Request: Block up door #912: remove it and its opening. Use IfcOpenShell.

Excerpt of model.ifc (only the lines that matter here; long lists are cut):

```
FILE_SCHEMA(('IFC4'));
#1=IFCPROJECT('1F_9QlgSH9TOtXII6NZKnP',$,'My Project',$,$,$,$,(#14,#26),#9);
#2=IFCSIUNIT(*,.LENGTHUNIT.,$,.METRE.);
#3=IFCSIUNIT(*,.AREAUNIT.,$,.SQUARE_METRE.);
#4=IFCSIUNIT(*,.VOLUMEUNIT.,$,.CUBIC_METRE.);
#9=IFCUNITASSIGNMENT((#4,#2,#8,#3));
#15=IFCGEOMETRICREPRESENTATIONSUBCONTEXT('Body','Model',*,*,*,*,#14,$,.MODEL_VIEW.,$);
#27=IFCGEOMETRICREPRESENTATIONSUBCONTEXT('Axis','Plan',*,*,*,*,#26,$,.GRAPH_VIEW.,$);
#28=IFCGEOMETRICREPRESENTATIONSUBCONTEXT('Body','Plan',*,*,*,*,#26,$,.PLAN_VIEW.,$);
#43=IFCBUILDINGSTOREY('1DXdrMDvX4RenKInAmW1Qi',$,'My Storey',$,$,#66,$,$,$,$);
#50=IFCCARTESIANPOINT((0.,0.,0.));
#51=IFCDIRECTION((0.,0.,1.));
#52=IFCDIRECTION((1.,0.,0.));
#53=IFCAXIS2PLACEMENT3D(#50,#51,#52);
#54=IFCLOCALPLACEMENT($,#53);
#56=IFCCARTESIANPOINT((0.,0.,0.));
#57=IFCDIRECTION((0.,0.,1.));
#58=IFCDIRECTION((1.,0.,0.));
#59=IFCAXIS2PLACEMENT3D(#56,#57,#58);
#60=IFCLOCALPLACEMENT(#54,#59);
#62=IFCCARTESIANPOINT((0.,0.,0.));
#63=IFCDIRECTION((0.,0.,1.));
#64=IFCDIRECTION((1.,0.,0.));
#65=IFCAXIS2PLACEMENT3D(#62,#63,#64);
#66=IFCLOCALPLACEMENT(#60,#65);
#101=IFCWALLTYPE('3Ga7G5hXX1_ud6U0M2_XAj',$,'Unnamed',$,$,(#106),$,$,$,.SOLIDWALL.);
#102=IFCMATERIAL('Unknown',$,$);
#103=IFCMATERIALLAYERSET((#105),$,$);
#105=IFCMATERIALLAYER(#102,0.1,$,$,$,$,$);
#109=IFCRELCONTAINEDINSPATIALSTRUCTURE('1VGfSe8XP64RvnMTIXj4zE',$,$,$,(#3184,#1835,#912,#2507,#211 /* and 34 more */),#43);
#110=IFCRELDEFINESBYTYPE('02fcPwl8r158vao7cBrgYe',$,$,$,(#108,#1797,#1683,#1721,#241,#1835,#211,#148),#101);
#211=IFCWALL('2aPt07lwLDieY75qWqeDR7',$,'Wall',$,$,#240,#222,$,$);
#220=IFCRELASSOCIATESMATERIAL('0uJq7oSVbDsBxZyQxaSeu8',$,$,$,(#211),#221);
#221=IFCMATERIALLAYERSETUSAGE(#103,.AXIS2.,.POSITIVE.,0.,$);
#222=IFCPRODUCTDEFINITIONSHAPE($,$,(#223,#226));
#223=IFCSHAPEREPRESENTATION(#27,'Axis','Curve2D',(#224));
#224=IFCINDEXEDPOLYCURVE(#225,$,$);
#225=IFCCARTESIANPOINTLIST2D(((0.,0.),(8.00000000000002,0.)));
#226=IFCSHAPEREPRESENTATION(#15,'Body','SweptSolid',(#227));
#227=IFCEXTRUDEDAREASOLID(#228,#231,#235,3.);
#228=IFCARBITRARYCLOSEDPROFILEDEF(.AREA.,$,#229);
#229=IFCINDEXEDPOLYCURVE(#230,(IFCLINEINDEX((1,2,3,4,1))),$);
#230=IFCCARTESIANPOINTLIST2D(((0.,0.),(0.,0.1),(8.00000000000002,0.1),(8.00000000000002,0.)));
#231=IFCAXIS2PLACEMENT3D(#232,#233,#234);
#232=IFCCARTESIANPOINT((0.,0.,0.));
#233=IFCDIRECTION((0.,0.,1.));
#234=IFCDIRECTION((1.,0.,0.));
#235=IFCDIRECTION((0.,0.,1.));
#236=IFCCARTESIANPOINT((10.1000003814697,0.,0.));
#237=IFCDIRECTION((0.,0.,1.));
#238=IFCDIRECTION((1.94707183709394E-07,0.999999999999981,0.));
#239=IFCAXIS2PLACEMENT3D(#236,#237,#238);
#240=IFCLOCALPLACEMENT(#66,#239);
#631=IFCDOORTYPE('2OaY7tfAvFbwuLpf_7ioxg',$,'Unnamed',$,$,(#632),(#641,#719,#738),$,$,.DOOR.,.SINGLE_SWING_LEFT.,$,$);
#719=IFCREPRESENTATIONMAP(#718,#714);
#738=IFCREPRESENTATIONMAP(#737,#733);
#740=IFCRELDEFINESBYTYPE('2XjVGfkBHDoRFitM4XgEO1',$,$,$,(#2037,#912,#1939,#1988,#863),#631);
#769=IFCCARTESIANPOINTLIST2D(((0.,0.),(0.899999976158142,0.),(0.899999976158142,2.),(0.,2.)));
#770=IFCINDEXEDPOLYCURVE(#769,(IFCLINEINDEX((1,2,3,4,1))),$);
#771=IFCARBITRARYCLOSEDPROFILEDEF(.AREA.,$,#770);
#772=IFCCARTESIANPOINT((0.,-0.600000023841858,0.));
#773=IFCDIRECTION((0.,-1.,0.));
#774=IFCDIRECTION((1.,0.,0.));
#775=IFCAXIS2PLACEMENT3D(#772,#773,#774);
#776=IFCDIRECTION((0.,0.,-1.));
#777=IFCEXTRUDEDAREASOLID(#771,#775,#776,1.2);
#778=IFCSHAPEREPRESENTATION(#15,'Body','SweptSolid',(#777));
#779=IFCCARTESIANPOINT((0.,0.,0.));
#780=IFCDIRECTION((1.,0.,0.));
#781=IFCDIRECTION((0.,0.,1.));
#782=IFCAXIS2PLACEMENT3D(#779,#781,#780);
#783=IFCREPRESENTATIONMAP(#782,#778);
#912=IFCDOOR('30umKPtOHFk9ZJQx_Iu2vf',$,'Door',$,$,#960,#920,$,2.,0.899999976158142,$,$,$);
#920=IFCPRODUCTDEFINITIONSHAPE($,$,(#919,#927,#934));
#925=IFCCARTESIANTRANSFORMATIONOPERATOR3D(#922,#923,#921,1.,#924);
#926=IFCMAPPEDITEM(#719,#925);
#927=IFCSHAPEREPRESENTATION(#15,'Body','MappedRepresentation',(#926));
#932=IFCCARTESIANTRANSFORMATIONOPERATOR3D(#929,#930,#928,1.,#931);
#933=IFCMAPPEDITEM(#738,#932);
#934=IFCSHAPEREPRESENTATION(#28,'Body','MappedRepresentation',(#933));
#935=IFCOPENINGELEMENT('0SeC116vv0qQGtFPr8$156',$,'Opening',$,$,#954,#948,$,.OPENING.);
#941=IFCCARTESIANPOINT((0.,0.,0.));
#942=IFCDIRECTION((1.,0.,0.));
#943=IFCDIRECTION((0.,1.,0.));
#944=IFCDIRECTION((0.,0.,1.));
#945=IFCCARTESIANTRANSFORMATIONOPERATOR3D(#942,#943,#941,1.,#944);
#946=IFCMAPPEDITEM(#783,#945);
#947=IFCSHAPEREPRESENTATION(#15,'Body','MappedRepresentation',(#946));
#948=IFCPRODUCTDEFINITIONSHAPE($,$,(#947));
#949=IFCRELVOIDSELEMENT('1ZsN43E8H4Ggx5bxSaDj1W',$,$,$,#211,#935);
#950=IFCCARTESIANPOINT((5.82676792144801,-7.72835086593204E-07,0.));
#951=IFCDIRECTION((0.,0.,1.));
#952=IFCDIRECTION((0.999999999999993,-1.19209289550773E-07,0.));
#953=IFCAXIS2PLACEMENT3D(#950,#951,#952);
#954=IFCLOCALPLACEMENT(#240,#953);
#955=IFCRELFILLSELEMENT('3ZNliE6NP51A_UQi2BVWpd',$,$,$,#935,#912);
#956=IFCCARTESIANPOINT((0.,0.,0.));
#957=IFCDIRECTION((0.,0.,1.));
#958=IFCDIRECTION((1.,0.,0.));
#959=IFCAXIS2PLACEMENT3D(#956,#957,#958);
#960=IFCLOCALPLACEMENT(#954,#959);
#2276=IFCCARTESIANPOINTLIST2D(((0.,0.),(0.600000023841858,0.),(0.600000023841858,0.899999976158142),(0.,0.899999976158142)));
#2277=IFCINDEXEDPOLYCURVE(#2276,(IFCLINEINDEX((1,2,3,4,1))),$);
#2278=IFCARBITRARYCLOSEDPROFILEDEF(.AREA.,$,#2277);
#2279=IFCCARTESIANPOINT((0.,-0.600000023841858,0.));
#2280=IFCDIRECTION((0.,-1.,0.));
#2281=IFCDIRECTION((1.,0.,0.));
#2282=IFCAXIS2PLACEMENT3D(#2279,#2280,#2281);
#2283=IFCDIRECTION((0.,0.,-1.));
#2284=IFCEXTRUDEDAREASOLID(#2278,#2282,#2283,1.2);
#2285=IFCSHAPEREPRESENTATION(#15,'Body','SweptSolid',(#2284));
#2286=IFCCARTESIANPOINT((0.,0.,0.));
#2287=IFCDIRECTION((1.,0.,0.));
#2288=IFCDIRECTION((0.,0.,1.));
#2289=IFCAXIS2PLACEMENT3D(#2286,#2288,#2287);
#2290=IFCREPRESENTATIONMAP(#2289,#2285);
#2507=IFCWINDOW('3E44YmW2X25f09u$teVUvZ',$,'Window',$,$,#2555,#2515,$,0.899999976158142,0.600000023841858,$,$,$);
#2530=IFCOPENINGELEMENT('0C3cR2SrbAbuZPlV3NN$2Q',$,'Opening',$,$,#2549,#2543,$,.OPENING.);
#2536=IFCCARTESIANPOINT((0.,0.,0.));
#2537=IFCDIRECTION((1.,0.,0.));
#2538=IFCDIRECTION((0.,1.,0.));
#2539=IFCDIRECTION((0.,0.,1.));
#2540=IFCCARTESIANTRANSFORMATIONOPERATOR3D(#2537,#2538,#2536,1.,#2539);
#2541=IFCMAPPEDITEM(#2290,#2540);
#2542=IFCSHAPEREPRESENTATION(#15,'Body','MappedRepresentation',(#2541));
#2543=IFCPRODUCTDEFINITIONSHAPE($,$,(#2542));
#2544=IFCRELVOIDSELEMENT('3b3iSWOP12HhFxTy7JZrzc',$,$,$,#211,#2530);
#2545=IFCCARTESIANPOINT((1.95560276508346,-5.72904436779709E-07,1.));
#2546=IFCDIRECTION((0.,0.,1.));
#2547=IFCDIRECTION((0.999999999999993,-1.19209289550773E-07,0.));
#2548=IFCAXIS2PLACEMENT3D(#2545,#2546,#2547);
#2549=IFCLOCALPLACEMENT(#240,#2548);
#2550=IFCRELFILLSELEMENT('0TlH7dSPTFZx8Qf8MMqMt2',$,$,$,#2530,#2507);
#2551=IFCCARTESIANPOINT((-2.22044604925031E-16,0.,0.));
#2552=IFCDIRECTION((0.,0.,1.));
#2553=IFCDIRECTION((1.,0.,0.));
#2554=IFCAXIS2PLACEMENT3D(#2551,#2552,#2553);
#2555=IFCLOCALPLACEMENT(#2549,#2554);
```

```python
import ifcopenshell
import ifcopenshell.api.feature
import ifcopenshell.api.root
import ifcopenshell.geom
import ifcopenshell.util.shape

model = ifcopenshell.open("model.ifc")
settings = ifcopenshell.geom.settings()


def volume(element):
    """Net volume in cubic metres, openings subtracted."""
    shape = ifcopenshell.geom.create_shape(settings, element)
    return ifcopenshell.util.shape.get_volume(shape.geometry)


door = model.by_guid("30umKPtOHFk9ZJQx_Iu2vf")
opening = door.FillsVoids[0].RelatingOpeningElement
wall = opening.VoidsElements[0].RelatingBuildingElement
before = volume(wall)

ifcopenshell.api.root.remove_product(model, product=door)
ifcopenshell.api.feature.remove_feature(model, feature=opening)

after = volume(wall)

print(f"wall volume {before:.3f} -> {after:.3f} m3")

model.write("model_v2.ifc")
```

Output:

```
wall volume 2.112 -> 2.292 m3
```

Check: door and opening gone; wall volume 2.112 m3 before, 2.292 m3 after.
